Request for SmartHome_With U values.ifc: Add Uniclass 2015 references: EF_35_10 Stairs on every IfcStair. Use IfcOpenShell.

First a look at what the model holds.

```python
import ifcopenshell

model = ifcopenshell.open("SmartHome_With U values.ifc")
print(model.schema)
print("classifications:", [c.Name for c in model.by_type("IfcClassification")])
for ifc_class in ("IfcDoor", "IfcRoof", "IfcStair", "IfcWall", "IfcWindow"):
    print(ifc_class, len(model.by_type(ifc_class)))
```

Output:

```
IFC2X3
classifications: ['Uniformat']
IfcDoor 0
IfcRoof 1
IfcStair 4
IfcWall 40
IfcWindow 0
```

```python
import ifcopenshell
import ifcopenshell.api.classification

model = ifcopenshell.open("SmartHome_With U values.ifc")

# IFC2X3 requires Source and Edition and has no link from the project to the system.
system = model.create_entity("IfcClassification", Source="NBS", Edition="2015", Name="Uniclass 2015")

codes = {
    "IfcStair": ("EF_35_10", "Stairs"),
}
for ifc_class, (code, name) in codes.items():
    products = model.by_type(ifc_class)
    ifcopenshell.api.classification.add_reference(
        model, products=products, classification=system, identification=code, name=name
    )
    print(code, len(products))

model.write("SmartHome_With U values_v2.ifc")
```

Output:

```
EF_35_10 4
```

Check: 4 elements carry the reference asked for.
